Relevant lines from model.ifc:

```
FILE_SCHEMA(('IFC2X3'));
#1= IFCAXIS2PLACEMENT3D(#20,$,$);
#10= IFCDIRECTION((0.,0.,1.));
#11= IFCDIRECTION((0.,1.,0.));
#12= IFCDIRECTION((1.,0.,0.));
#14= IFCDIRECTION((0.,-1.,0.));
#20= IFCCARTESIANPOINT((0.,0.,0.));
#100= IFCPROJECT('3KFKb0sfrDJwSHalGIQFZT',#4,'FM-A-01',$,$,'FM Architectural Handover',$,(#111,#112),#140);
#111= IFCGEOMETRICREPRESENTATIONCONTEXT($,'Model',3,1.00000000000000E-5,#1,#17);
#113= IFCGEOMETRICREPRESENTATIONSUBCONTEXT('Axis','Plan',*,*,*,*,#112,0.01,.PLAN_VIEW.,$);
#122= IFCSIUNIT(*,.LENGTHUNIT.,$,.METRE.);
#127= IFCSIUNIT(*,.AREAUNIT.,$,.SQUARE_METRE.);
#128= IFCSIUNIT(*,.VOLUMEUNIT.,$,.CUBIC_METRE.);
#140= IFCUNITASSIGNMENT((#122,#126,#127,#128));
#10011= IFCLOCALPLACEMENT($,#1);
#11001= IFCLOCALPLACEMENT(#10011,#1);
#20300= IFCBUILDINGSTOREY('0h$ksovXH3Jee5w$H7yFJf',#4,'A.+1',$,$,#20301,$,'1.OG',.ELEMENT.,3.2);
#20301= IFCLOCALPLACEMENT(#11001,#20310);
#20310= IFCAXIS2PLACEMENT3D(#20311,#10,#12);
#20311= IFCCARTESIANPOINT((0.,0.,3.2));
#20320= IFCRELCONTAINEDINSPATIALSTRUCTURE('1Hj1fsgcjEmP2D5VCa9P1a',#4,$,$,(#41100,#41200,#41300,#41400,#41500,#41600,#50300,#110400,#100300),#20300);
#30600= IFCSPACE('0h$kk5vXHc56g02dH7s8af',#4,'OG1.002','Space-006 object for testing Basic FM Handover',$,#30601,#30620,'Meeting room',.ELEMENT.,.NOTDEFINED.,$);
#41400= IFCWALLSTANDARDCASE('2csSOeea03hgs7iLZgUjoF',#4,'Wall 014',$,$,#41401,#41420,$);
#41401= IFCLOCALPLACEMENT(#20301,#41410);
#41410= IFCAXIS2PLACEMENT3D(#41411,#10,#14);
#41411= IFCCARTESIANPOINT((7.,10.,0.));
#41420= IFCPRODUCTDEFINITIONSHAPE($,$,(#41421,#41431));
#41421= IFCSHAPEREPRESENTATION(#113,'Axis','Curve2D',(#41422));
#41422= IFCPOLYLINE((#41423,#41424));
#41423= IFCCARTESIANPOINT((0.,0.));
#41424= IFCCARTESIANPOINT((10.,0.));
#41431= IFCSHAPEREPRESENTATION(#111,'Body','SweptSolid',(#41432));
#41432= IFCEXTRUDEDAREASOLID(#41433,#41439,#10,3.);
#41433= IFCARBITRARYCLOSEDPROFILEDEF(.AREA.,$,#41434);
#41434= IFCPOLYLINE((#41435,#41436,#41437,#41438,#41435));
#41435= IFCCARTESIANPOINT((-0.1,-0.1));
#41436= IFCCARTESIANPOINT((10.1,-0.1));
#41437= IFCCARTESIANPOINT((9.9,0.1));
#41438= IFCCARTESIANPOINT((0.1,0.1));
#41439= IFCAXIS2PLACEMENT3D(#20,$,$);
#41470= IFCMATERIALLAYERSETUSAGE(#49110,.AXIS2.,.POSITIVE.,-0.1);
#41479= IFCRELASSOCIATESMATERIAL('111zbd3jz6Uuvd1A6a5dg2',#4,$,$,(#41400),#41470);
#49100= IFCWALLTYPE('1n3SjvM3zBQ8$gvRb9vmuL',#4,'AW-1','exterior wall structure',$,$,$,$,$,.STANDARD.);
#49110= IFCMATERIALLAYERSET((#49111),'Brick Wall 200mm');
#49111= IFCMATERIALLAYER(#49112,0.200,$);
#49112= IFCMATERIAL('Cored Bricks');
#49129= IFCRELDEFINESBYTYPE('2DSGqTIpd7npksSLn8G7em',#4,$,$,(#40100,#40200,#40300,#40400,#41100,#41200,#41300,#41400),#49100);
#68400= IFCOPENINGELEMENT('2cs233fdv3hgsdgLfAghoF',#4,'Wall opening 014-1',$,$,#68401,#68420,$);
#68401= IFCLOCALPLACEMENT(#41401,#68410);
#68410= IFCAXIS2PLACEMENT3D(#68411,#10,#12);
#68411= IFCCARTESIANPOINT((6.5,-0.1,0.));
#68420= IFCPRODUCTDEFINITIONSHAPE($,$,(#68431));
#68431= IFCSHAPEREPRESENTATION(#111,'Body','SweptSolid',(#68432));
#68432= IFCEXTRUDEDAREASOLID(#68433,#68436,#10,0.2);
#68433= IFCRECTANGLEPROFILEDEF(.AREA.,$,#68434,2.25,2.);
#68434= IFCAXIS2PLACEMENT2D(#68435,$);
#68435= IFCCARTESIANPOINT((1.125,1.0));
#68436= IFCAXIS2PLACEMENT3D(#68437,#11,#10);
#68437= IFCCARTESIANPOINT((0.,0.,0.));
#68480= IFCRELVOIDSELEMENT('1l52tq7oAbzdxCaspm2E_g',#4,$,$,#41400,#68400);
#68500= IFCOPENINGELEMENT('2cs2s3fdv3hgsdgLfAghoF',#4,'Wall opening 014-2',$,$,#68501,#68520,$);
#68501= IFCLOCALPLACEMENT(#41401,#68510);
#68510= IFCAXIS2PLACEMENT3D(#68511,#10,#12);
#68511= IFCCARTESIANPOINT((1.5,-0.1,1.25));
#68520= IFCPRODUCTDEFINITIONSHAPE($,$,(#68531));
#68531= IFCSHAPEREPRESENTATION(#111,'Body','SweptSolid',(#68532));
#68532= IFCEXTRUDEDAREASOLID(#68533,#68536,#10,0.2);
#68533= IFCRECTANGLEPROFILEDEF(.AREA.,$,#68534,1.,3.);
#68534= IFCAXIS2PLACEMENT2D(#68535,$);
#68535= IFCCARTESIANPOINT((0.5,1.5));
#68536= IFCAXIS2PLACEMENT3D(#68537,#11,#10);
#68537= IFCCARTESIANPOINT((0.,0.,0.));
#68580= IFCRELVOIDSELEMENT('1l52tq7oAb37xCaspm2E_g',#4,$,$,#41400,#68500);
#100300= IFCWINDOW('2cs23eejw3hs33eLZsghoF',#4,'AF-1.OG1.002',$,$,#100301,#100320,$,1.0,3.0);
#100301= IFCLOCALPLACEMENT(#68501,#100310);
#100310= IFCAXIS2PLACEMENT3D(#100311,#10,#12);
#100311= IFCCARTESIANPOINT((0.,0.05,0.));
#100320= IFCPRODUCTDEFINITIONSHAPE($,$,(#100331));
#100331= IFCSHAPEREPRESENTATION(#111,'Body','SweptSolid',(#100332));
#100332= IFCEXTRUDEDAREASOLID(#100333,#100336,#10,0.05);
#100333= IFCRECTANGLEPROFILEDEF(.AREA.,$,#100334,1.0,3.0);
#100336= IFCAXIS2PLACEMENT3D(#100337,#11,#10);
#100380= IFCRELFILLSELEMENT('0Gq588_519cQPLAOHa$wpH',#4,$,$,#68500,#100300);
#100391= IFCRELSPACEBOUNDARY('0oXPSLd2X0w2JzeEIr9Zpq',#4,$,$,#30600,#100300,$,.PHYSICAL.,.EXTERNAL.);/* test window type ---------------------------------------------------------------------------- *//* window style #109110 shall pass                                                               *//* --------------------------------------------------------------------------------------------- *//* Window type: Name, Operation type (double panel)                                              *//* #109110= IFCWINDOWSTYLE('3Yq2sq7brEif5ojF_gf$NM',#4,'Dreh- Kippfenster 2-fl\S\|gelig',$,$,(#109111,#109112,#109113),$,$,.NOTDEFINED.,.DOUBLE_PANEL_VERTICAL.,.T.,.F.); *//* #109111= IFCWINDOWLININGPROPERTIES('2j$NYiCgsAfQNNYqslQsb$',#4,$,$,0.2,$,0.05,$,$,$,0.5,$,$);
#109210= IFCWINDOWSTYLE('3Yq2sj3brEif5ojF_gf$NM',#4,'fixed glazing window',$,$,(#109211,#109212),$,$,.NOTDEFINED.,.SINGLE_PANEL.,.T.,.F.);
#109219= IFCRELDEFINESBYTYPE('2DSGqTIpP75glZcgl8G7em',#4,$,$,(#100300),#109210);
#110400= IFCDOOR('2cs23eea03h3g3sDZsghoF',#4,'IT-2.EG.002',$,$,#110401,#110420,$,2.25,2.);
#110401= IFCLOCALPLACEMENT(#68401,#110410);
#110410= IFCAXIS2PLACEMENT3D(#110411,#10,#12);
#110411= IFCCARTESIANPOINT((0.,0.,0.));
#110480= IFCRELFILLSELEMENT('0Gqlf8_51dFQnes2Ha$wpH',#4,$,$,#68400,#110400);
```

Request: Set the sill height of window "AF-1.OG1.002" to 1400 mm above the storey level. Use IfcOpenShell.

```python
import numpy as np
import ifcopenshell
import ifcopenshell.api.geometry
import ifcopenshell.geom
import ifcopenshell.util.element
import ifcopenshell.util.placement
import ifcopenshell.util.shape
import ifcopenshell.util.unit

model = ifcopenshell.open("model.ifc")
unit_scale = ifcopenshell.util.unit.calculate_unit_scale(model)

window = model.by_guid("2cs23eejw3hs33eLZsghoF")
opening = window.FillsVoids[0].RelatingOpeningElement
storey = ifcopenshell.util.element.get_container(window, ifc_class="IfcBuildingStorey")
level = ifcopenshell.util.placement.get_local_placement(storey.ObjectPlacement)[2, 3]

# The opening's origin need not be at the sill, so measure its lowest point.
shape = ifcopenshell.geom.create_shape(ifcopenshell.geom.settings(), opening)
bottom = ifcopenshell.util.shape.get_shape_bottom_elevation(shape, shape.geometry) / unit_scale
dz = level + 1.4 - bottom

shift = np.array([0.0, 0.0, dz])
# The window is placed relative to its opening, so it follows when the opening moves.
matrix = ifcopenshell.util.placement.get_local_placement(opening.ObjectPlacement)
matrix[:3, 3] += shift
ifcopenshell.api.geometry.edit_object_placement(
    model, product=opening, matrix=matrix, is_si=False, should_transform_children=True
)

print(f"moved by {dz * unit_scale:+.3f} m")

model.write("model_rev.ifc")
```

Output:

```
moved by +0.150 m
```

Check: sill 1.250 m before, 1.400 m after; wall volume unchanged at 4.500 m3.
